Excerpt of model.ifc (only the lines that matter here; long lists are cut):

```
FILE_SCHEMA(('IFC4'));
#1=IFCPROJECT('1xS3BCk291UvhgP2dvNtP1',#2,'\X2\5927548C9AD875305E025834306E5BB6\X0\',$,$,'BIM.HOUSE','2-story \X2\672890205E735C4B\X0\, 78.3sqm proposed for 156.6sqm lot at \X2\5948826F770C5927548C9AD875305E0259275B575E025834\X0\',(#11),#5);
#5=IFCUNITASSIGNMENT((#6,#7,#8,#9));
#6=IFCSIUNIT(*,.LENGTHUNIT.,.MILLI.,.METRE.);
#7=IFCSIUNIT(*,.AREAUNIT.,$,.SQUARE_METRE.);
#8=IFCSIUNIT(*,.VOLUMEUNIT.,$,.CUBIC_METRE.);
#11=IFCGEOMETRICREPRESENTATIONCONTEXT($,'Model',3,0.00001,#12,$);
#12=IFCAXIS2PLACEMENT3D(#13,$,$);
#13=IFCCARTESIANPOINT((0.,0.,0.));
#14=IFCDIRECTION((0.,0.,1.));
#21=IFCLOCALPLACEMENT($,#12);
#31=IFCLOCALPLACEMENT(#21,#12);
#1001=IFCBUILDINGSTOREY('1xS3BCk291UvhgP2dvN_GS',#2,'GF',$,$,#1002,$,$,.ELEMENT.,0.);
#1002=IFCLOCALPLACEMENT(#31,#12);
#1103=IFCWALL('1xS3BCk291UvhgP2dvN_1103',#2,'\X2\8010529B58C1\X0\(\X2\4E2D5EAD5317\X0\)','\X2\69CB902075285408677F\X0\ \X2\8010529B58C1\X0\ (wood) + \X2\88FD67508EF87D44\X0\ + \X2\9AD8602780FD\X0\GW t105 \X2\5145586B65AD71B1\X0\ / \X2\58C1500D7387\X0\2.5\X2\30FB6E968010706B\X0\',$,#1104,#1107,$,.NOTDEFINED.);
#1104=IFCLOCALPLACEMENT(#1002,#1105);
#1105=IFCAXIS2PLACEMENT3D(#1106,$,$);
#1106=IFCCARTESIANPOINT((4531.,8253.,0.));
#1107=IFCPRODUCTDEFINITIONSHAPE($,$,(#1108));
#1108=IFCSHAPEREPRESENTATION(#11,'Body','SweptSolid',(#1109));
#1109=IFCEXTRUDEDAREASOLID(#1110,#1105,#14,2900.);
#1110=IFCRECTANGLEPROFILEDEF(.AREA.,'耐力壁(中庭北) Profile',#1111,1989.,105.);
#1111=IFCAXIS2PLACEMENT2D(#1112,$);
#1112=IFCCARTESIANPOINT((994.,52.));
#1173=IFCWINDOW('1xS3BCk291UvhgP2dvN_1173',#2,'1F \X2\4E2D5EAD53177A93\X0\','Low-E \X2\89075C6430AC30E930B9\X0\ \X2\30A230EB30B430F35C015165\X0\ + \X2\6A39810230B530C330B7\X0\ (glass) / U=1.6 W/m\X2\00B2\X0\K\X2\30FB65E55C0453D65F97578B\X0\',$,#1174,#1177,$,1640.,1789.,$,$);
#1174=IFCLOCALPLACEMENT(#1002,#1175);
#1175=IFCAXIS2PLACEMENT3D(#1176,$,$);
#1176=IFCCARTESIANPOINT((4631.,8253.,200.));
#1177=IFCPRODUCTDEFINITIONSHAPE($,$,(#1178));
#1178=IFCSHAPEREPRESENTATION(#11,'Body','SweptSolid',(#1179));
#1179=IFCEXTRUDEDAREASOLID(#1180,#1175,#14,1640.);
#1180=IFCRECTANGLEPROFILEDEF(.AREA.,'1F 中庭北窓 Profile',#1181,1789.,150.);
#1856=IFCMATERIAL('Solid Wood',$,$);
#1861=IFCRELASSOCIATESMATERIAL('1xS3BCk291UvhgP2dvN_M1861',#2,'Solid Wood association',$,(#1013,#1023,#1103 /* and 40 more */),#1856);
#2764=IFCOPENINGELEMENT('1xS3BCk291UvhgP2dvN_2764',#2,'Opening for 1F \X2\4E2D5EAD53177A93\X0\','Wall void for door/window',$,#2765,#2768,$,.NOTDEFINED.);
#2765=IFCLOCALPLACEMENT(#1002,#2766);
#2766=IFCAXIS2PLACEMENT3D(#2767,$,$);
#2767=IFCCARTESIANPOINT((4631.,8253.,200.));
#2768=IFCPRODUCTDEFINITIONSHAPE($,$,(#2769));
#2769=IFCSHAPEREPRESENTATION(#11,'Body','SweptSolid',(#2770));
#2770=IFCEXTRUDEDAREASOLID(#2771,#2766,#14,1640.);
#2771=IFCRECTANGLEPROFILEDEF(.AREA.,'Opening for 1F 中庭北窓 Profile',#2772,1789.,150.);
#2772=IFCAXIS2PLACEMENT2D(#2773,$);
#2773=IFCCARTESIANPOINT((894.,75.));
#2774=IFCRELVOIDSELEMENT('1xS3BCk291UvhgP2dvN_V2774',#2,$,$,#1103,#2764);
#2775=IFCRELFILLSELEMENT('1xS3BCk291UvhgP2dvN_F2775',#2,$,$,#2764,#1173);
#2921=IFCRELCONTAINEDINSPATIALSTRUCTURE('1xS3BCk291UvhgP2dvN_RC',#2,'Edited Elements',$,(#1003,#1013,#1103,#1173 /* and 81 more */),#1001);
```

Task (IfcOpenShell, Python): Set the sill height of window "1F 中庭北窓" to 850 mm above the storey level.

```python
import numpy as np
import ifcopenshell
import ifcopenshell.api.geometry
import ifcopenshell.geom
import ifcopenshell.util.element
import ifcopenshell.util.placement
import ifcopenshell.util.shape
import ifcopenshell.util.unit

model = ifcopenshell.open("model.ifc")
unit_scale = ifcopenshell.util.unit.calculate_unit_scale(model)

window = model.by_id(1173)
opening = window.FillsVoids[0].RelatingOpeningElement
storey = ifcopenshell.util.element.get_container(window, ifc_class="IfcBuildingStorey")
level = ifcopenshell.util.placement.get_local_placement(storey.ObjectPlacement)[2, 3]

# The opening's origin need not be at the sill, so measure its lowest point.
shape = ifcopenshell.geom.create_shape(ifcopenshell.geom.settings(), opening)
bottom = ifcopenshell.util.shape.get_shape_bottom_elevation(shape, shape.geometry) / unit_scale
dz = level + 850.0 - bottom

shift = np.array([0.0, 0.0, dz])
# The window is not placed relative to its opening, so move both.
for product in (opening, window):
    matrix = ifcopenshell.util.placement.get_local_placement(product.ObjectPlacement)
    matrix[:3, 3] += shift
    ifcopenshell.api.geometry.edit_object_placement(model, product=product, matrix=matrix, is_si=False)

print(f"moved by {dz * unit_scale:+.3f} m")

model.write("model_v2.ifc")
```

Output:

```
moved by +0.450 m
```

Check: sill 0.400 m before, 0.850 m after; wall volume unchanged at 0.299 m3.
